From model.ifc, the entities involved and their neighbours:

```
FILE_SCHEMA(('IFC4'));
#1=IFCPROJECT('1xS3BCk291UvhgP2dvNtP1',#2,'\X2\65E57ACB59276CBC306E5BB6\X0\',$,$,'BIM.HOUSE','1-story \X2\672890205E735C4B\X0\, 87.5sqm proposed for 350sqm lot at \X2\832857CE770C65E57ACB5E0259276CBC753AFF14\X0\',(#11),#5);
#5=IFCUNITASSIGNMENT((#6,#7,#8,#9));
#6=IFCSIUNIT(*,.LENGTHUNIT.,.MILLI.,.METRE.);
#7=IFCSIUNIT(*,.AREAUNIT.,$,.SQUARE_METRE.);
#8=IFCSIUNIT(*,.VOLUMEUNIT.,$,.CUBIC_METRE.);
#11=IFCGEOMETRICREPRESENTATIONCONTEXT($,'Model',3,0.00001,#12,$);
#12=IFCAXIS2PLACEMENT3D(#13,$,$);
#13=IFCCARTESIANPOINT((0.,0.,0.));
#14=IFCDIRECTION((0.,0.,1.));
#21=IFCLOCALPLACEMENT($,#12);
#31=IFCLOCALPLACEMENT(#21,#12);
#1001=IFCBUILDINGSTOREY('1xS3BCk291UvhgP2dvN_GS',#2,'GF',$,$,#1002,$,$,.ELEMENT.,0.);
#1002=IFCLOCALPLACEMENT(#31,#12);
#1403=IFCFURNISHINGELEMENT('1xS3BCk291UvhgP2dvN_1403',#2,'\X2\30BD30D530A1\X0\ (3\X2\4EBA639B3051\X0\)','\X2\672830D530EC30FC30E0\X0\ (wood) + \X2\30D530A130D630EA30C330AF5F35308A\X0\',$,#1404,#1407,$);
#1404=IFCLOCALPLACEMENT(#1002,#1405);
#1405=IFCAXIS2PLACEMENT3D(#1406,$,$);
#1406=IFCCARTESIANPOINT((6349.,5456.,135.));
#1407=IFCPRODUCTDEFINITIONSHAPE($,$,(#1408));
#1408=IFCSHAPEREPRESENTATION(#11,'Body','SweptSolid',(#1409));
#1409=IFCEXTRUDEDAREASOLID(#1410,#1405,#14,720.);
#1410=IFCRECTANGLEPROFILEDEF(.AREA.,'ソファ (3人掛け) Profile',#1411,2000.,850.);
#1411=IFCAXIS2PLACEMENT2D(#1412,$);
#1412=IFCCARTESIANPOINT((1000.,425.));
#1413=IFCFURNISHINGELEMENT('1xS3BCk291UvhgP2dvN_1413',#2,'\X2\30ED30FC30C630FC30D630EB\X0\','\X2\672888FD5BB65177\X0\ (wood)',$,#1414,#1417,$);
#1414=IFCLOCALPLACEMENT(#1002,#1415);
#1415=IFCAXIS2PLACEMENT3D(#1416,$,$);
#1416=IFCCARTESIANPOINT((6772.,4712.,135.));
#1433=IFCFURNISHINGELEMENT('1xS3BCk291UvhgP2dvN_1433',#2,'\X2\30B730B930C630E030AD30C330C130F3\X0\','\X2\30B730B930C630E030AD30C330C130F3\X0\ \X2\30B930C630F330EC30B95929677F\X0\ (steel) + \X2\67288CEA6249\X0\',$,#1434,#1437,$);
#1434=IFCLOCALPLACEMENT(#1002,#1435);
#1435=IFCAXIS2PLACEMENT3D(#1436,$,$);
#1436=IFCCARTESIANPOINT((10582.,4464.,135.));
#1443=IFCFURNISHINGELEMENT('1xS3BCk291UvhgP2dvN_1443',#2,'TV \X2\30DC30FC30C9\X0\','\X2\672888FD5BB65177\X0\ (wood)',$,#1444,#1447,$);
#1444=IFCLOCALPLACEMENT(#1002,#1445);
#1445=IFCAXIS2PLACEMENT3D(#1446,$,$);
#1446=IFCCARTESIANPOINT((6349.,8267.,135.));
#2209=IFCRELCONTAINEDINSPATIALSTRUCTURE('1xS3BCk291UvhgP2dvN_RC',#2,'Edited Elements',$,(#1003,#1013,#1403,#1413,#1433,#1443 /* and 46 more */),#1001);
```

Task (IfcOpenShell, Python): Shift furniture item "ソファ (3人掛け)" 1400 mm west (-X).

```python
import ifcopenshell
import ifcopenshell.api.geometry
import ifcopenshell.util.placement

model = ifcopenshell.open("model.ifc")

item = model.by_guid("1xS3BCk291UvhgP2dvN_1403")
matrix = ifcopenshell.util.placement.get_local_placement(item.ObjectPlacement)
matrix[0, 3] -= 1400.0
ifcopenshell.api.geometry.edit_object_placement(model, product=item, matrix=matrix, is_si=False)

print(ifcopenshell.util.placement.get_local_placement(item.ObjectPlacement).round(3) + 0.0)

model.write("model_v2.ifc")
```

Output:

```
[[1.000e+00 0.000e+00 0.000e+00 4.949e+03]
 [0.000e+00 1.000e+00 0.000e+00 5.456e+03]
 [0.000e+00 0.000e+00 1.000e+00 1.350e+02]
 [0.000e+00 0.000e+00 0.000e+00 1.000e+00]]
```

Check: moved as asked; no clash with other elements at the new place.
